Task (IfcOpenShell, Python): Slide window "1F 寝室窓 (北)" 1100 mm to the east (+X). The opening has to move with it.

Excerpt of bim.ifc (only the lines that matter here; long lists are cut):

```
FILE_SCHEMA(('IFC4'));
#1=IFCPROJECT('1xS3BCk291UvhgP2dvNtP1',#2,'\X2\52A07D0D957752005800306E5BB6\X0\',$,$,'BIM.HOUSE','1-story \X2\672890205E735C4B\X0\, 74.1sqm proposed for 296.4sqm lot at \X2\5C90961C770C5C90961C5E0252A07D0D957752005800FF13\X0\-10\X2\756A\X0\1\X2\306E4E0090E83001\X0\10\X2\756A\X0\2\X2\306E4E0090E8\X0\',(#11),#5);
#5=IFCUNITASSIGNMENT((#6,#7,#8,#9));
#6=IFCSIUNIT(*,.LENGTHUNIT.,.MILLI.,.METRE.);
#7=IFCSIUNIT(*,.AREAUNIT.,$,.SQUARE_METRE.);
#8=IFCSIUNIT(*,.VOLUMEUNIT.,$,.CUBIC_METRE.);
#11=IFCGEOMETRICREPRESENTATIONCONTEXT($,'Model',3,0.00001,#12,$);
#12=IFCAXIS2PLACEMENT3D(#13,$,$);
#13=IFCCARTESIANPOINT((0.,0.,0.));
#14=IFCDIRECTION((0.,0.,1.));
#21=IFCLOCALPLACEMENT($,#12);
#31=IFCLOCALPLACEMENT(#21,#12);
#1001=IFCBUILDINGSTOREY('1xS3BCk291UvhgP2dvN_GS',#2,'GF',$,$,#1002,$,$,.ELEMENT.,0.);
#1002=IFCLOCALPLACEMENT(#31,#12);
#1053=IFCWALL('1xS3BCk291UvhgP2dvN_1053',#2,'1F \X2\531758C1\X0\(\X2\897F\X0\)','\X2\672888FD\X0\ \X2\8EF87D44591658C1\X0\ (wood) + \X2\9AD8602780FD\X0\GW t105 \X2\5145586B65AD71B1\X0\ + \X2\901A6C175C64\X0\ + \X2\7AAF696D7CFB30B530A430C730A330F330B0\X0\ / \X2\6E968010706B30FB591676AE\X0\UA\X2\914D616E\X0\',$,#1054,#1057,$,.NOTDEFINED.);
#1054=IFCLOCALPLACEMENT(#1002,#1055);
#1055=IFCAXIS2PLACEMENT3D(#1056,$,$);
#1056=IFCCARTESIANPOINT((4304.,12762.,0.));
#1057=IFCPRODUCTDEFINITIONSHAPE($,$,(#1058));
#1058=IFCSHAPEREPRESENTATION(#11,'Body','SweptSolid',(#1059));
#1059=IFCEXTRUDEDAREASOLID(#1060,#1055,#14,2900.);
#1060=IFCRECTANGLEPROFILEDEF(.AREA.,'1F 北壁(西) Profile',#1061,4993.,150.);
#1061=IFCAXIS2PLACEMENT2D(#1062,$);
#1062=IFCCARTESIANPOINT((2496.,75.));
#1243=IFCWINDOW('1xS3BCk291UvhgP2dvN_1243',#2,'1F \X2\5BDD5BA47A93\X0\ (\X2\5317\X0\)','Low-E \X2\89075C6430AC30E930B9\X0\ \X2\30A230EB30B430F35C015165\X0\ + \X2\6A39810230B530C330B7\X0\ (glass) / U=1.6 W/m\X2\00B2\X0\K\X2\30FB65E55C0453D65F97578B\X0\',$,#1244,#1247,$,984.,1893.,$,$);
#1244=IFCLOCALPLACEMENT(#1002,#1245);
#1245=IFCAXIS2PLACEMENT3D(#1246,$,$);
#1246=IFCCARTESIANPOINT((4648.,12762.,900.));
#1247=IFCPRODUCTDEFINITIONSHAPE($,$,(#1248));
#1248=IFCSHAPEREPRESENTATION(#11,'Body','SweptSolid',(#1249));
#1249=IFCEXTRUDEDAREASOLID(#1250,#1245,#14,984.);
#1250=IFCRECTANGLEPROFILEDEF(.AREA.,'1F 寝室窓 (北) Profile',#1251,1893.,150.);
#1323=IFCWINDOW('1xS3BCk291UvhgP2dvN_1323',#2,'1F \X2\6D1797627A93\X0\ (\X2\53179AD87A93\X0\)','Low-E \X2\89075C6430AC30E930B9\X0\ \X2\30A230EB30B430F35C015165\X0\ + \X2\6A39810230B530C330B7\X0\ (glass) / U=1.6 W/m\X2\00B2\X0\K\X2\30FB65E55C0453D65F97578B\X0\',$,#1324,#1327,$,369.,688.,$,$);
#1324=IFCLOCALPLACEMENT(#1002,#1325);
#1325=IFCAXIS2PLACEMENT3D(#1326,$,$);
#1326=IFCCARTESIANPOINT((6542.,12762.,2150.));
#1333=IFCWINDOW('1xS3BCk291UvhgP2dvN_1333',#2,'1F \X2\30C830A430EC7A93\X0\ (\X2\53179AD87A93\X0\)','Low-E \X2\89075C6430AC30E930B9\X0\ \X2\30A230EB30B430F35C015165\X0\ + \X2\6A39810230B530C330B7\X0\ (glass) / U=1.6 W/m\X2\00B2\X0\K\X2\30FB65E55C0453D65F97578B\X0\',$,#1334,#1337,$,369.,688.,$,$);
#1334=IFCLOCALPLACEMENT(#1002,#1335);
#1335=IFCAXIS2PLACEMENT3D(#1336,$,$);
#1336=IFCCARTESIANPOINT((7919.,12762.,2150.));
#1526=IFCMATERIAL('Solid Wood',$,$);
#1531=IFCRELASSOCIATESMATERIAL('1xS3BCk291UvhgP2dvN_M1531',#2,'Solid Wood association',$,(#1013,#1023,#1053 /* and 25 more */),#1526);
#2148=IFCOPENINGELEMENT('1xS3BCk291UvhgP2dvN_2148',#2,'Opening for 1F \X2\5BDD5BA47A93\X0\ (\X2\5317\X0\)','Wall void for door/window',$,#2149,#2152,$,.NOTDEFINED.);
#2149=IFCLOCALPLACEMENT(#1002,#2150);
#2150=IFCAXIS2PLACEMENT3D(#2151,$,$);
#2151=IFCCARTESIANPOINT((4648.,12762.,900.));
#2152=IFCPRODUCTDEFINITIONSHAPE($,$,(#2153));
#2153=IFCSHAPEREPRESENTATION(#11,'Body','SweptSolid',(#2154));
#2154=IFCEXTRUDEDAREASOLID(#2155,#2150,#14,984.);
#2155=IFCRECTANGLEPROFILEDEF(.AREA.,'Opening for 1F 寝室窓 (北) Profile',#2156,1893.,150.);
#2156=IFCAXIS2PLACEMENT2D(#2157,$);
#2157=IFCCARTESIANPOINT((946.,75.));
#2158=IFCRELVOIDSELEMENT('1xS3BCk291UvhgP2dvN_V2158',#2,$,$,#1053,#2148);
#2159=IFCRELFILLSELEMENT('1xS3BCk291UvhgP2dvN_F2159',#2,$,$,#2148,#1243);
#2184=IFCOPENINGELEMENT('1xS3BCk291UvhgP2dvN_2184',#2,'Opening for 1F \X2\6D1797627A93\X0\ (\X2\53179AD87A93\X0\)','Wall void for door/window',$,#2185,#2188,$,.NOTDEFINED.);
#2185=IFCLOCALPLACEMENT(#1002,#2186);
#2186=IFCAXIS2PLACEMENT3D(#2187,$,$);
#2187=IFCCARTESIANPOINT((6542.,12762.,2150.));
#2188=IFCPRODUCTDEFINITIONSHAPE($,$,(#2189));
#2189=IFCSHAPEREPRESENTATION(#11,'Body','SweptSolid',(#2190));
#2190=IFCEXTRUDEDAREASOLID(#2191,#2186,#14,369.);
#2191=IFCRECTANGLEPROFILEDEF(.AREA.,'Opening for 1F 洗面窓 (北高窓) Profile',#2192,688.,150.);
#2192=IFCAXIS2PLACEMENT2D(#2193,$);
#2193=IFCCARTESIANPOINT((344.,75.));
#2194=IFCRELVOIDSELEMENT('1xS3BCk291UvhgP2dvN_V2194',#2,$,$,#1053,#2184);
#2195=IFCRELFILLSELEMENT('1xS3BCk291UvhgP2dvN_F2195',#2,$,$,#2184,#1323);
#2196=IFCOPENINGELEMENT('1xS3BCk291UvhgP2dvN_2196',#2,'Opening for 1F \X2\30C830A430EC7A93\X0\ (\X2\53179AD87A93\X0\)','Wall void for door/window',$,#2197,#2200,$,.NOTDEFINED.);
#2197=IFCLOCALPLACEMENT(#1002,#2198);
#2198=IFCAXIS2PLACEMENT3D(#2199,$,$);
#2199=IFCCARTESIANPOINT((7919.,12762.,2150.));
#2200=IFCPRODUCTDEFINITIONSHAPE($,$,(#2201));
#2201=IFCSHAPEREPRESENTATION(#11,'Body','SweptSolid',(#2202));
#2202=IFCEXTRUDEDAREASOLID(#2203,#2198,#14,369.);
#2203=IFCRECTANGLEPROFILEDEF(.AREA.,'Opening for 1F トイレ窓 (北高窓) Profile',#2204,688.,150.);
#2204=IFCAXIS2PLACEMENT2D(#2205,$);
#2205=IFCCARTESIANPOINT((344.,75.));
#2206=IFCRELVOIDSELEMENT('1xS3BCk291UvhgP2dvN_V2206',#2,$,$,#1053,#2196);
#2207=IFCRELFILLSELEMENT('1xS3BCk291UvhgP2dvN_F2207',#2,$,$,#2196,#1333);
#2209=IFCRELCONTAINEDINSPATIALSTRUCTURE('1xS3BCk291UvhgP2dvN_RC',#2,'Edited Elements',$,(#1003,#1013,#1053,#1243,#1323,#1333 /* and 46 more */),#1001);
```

```python
import ifcopenshell
import ifcopenshell.api.geometry
import ifcopenshell.util.placement
import ifcopenshell.util.unit

model = ifcopenshell.open("bim.ifc")
unit_scale = ifcopenshell.util.unit.calculate_unit_scale(model)

window = model.by_guid("1xS3BCk291UvhgP2dvN_1243")
opening = window.FillsVoids[0].RelatingOpeningElement
wall = opening.VoidsElements[0].RelatingBuildingElement

wall_matrix = ifcopenshell.util.placement.get_local_placement(wall.ObjectPlacement)
shift = wall_matrix[:3, 0] * 1.1 / unit_scale
before = ifcopenshell.util.placement.get_local_placement(window.ObjectPlacement)[:3, 3].copy()

# The window is not placed relative to its opening, so move both.
for product in (opening, window):
    matrix = ifcopenshell.util.placement.get_local_placement(product.ObjectPlacement)
    matrix[:3, 3] += shift
    ifcopenshell.api.geometry.edit_object_placement(model, product=product, matrix=matrix, is_si=False)

after = ifcopenshell.util.placement.get_local_placement(window.ObjectPlacement)[:3, 3]
print("window moved by", (after - before).round(3) + 0.0)

model.write("bim_edited.ifc")
```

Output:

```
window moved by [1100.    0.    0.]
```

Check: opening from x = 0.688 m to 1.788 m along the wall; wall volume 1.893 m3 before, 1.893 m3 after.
